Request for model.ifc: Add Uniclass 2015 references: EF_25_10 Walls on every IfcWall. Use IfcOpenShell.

First a look at what the model holds.

```python
import ifcopenshell

model = ifcopenshell.open("model.ifc")
print(model.schema)
print("classifications:", [c.Name for c in model.by_type("IfcClassification")])
for ifc_class in ("IfcDoor", "IfcRoof", "IfcStair", "IfcWall", "IfcWindow"):
    print(ifc_class, len(model.by_type(ifc_class)))
```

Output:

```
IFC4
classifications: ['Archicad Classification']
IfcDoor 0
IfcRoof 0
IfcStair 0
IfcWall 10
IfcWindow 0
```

```python
import ifcopenshell
import ifcopenshell.api.classification

model = ifcopenshell.open("model.ifc")

system = ifcopenshell.api.classification.add_classification(model, classification="Uniclass 2015")

codes = {
    "IfcWall": ("EF_25_10", "Walls"),
}
for ifc_class, (code, name) in codes.items():
    products = model.by_type(ifc_class)
    ifcopenshell.api.classification.add_reference(
        model, products=products, classification=system, identification=code, name=name
    )
    print(code, len(products))

model.write("model_v2.ifc")
```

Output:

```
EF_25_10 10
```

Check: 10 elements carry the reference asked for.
